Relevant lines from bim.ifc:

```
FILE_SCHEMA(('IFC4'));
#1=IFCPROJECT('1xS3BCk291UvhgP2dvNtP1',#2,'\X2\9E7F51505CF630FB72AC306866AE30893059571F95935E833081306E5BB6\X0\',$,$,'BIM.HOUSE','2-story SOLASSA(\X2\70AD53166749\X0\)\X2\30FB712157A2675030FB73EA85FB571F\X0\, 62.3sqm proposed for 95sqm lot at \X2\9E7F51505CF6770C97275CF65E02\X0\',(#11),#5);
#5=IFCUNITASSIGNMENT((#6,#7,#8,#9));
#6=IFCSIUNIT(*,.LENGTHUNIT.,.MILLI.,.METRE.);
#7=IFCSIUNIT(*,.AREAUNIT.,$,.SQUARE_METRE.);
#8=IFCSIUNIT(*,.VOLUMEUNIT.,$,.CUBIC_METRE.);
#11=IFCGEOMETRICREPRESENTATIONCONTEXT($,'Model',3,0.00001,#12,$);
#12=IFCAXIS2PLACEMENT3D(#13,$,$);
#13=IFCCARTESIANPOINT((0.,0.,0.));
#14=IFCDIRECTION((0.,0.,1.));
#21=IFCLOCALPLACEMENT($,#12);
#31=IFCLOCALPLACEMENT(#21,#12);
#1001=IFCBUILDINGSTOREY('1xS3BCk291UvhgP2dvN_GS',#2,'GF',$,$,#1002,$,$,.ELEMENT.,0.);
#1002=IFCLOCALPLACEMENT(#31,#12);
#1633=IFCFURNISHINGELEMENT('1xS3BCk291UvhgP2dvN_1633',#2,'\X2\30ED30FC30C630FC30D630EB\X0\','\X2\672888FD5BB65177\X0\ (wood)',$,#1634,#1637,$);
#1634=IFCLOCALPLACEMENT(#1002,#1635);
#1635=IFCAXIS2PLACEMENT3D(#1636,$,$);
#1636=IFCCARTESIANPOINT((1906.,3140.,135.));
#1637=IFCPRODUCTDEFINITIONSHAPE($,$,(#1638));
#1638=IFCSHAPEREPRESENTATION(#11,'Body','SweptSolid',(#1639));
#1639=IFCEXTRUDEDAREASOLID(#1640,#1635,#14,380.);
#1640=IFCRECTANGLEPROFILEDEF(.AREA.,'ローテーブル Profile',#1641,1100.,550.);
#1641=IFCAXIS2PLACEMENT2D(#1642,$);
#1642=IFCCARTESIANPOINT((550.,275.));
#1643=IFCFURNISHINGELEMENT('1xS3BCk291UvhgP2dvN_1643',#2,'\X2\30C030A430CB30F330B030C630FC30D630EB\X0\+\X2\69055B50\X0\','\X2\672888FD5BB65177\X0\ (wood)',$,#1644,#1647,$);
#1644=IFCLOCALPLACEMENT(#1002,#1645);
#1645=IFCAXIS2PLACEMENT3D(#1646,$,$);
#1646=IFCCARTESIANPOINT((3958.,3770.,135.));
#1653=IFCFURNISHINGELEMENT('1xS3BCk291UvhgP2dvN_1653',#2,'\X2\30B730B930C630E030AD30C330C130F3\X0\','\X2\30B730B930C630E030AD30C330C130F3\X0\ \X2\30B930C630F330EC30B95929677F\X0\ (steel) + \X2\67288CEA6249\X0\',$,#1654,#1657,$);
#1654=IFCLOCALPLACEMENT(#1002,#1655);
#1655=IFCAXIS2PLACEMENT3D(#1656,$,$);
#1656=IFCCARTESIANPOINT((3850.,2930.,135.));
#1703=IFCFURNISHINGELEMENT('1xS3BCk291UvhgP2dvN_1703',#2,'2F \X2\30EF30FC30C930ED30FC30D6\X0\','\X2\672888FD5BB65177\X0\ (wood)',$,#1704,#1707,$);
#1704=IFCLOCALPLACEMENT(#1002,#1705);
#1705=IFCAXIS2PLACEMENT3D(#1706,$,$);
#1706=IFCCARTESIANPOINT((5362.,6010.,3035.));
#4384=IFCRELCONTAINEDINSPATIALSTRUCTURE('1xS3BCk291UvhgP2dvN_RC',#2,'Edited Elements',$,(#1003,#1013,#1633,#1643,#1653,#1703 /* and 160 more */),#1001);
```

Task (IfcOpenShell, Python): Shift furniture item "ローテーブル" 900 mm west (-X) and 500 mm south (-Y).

```python
import ifcopenshell
import ifcopenshell.api.geometry
import ifcopenshell.util.placement
import ifcopenshell.util.unit

model = ifcopenshell.open("bim.ifc")
unit_scale = ifcopenshell.util.unit.calculate_unit_scale(model)

item = model.by_id(1633)
matrix = ifcopenshell.util.placement.get_local_placement(item.ObjectPlacement)
matrix[0, 3] -= 0.9 / unit_scale
matrix[1, 3] -= 0.5 / unit_scale
ifcopenshell.api.geometry.edit_object_placement(model, product=item, matrix=matrix, is_si=False)

print(ifcopenshell.util.placement.get_local_placement(item.ObjectPlacement).round(3) + 0.0)

model.write("bim_updated.ifc")
```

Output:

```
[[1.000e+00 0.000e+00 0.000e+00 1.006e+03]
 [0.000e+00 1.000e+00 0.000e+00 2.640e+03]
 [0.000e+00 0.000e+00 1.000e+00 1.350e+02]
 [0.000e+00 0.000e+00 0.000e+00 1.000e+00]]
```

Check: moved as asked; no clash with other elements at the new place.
